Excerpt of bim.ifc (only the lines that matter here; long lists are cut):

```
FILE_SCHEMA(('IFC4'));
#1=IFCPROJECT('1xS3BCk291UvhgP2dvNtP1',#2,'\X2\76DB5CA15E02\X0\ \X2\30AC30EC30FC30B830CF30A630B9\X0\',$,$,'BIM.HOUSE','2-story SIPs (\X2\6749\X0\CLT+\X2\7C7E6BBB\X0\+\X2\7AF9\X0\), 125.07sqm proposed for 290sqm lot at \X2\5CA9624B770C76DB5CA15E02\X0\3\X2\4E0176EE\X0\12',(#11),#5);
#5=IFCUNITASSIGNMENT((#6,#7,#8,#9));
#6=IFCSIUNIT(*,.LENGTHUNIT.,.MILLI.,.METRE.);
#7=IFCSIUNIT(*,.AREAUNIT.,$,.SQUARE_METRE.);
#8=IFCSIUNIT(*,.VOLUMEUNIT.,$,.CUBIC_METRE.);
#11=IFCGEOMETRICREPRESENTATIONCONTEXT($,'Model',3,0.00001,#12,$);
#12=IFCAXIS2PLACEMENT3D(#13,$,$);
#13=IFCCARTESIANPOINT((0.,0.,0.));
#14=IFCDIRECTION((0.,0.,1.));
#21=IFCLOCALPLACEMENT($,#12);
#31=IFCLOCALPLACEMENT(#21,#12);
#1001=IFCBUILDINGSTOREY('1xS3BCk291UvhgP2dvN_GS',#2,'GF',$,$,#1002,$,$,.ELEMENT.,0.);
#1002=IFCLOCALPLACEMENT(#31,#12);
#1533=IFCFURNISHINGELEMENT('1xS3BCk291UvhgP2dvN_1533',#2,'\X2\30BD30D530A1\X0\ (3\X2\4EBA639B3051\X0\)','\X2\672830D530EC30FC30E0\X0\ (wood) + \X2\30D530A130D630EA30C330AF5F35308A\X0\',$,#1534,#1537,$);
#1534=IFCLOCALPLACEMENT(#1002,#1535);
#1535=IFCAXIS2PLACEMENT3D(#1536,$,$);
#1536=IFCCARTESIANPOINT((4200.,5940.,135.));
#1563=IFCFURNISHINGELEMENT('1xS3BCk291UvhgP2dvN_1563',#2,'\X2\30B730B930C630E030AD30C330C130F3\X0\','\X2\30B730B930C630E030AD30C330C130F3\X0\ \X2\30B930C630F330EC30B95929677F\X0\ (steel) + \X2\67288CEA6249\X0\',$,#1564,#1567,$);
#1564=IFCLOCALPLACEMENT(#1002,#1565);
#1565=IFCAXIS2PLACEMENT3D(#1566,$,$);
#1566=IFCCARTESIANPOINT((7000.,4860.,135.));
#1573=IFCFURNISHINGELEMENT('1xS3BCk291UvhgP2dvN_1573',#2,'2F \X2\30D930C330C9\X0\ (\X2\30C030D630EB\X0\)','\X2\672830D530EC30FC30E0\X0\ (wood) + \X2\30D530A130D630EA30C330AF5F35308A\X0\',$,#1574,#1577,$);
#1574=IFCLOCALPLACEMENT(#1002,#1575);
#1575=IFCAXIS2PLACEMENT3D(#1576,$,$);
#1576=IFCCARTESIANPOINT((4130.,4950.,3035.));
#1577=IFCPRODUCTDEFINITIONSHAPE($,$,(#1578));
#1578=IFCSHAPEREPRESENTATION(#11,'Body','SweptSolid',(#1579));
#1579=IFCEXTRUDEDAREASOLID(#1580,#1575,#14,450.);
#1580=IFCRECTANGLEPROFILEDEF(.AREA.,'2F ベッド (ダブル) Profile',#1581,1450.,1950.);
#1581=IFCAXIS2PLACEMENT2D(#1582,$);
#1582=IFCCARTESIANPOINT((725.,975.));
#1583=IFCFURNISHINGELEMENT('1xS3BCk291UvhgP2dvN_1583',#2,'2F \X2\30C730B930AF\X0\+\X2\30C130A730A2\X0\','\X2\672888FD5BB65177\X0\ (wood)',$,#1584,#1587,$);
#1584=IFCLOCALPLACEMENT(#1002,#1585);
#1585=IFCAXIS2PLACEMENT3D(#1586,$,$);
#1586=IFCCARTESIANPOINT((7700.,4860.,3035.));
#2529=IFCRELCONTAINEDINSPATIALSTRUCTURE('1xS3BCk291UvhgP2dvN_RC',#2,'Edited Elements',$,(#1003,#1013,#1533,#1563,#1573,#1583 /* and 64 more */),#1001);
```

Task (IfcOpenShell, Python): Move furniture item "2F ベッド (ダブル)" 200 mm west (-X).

```python
import ifcopenshell
import ifcopenshell.api.geometry
import ifcopenshell.util.placement
import ifcopenshell.util.unit

model = ifcopenshell.open("bim.ifc")
unit_scale = ifcopenshell.util.unit.calculate_unit_scale(model)

item = model.by_guid("1xS3BCk291UvhgP2dvN_1573")
matrix = ifcopenshell.util.placement.get_local_placement(item.ObjectPlacement)
matrix[0, 3] -= 0.2 / unit_scale
ifcopenshell.api.geometry.edit_object_placement(model, product=item, matrix=matrix, is_si=False)

print(ifcopenshell.util.placement.get_local_placement(item.ObjectPlacement).round(3) + 0.0)

model.write("bim-out.ifc")
```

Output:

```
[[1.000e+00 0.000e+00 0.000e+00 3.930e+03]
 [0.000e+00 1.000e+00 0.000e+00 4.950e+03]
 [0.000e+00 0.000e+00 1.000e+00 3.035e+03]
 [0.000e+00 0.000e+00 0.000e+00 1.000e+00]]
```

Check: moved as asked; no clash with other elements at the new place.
